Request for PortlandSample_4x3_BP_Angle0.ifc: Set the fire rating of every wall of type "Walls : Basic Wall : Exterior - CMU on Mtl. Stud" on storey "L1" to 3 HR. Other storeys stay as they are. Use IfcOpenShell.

First a look at what the model holds.

```python
import ifcopenshell
import ifcopenshell.util.element

model = ifcopenshell.open("PortlandSample_4x3_BP_Angle0.ifc")
print(model.schema)
storey = next(s for s in model.by_type("IfcBuildingStorey") if s.Name == "L1")
walls = [e for e in ifcopenshell.util.element.get_decomposition(storey) if e.is_a("IfcWall")]
seen = {}
for e in walls:
    element_type = ifcopenshell.util.element.get_type(e)
    key = (element_type.Name if element_type != e and element_type else None, ifcopenshell.util.element.get_pset(e, "Pset_WallCommon", "FireRating"))
    seen[key] = seen.get(key, 0) + 1
for (name, value), count in sorted(seen.items(), key=str):
    print(count, "x", name, "|", value)
```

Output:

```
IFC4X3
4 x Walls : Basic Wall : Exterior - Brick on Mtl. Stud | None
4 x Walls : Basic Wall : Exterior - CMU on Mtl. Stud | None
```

```python
import ifcopenshell
import ifcopenshell.api.pset
import ifcopenshell.util.element

model = ifcopenshell.open("PortlandSample_4x3_BP_Angle0.ifc")

storey = next(s for s in model.by_type("IfcBuildingStorey") if s.Name == "L1")
walls = [e for e in ifcopenshell.util.element.get_decomposition(storey) if e.is_a("IfcWall")]

count = 0
for e in walls:
    element_type = ifcopenshell.util.element.get_type(e)
    if element_type in (None, e) or element_type.Name != "Walls : Basic Wall : Exterior - CMU on Mtl. Stud":
        continue
    # add_pset returns the element's existing set when there is one.
    pset = ifcopenshell.api.pset.add_pset(model, product=e, name="Pset_WallCommon")
    ifcopenshell.api.pset.edit_pset(model, pset=pset, properties={"FireRating": "3 HR"})
    count += 1

print(count, "walls updated")

model.write("PortlandSample_4x3_BP_Angle0_updated.ifc")
```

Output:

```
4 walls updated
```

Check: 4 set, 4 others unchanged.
